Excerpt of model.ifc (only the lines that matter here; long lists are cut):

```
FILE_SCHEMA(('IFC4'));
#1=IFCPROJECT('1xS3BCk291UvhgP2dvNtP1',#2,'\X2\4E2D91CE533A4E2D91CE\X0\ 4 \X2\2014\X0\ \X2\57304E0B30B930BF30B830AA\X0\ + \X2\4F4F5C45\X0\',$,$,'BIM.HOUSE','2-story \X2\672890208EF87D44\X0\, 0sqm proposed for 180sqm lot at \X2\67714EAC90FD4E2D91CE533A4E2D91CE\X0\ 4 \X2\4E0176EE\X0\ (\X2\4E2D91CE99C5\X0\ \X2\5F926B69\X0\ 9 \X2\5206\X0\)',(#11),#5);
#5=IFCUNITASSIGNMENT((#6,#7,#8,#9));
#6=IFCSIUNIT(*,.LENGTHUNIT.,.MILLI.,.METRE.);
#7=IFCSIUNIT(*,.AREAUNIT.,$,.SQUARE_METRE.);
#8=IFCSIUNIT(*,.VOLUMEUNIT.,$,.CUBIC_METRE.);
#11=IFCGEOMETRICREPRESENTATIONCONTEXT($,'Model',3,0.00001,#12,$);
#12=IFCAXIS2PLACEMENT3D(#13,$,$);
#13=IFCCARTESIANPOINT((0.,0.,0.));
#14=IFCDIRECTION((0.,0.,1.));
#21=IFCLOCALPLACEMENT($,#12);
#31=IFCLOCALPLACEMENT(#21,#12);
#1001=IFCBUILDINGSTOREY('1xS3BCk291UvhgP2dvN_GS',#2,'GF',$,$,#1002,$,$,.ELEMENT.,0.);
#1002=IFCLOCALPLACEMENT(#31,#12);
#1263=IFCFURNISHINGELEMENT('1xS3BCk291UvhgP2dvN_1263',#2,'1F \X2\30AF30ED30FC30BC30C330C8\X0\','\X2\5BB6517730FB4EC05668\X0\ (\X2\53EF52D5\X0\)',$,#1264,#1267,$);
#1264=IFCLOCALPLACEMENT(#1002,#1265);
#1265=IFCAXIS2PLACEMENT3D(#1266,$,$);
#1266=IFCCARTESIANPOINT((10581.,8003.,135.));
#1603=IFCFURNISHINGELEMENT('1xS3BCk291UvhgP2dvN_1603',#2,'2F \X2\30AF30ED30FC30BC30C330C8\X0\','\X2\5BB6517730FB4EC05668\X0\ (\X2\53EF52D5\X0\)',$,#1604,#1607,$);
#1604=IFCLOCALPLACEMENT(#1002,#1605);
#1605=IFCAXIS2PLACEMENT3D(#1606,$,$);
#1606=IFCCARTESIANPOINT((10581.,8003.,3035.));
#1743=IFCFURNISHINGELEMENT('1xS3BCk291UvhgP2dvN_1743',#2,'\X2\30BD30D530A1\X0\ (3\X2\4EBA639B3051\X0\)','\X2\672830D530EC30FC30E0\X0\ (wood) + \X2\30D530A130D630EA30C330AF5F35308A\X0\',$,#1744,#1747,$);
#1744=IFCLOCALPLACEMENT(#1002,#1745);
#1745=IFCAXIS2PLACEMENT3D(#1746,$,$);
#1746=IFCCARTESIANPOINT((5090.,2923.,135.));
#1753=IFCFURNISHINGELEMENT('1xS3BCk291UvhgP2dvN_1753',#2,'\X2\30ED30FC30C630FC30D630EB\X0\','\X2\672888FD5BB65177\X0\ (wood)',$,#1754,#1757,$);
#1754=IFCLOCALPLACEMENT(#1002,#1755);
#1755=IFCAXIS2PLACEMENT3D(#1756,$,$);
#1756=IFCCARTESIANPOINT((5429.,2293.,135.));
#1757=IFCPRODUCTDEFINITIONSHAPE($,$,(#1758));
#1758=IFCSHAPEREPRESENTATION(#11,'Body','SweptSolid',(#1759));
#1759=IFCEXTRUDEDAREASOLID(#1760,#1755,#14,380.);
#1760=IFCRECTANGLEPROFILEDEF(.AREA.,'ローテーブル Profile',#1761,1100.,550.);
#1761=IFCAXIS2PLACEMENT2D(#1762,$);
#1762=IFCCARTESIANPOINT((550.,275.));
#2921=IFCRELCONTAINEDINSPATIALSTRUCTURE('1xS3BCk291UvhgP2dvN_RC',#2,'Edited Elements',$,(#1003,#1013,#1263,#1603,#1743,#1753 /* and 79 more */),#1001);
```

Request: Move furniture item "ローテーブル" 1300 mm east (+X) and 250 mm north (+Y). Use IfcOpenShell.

```python
import ifcopenshell
import ifcopenshell.api.geometry
import ifcopenshell.util.placement

model = ifcopenshell.open("model.ifc")

item = model.by_guid("1xS3BCk291UvhgP2dvN_1753")
matrix = ifcopenshell.util.placement.get_local_placement(item.ObjectPlacement)
matrix[0, 3] += 1300.0
matrix[1, 3] += 250.0
ifcopenshell.api.geometry.edit_object_placement(model, product=item, matrix=matrix, is_si=False)

print(ifcopenshell.util.placement.get_local_placement(item.ObjectPlacement).round(3) + 0.0)

model.write("model_edited.ifc")
```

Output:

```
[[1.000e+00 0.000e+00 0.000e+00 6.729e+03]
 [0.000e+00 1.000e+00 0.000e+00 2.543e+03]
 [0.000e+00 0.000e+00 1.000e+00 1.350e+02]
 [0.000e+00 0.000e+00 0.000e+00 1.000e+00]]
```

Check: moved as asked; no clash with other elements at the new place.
